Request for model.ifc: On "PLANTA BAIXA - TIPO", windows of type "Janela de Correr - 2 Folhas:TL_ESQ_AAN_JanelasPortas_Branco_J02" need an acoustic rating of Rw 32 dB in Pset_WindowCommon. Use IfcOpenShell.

First a look at what the model holds.

```python
import ifcopenshell
import ifcopenshell.util.element

model = ifcopenshell.open("model.ifc")
print(model.schema)
storey = next(s for s in model.by_type("IfcBuildingStorey") if s.Name == "PLANTA BAIXA - TIPO")
windows = [e for e in ifcopenshell.util.element.get_decomposition(storey) if e.is_a("IfcWindow")]
seen = {}
for e in windows:
    element_type = ifcopenshell.util.element.get_type(e)
    key = (element_type.Name if element_type != e and element_type else None, ifcopenshell.util.element.get_pset(e, "Pset_WindowCommon", "AcousticRating"))
    seen[key] = seen.get(key, 0) + 1
for (name, value), count in sorted(seen.items(), key=str):
    print(count, "x", name, "|", value)
```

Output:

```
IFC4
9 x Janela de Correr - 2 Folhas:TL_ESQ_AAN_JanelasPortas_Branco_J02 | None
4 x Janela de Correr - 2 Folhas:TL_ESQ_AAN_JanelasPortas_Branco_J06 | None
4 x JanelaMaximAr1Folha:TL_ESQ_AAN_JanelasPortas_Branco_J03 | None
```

```python
import ifcopenshell
import ifcopenshell.api.pset
import ifcopenshell.util.element

model = ifcopenshell.open("model.ifc")

storey = next(s for s in model.by_type("IfcBuildingStorey") if s.Name == "PLANTA BAIXA - TIPO")
windows = [e for e in ifcopenshell.util.element.get_decomposition(storey) if e.is_a("IfcWindow")]

count = 0
for e in windows:
    element_type = ifcopenshell.util.element.get_type(e)
    if element_type in (None, e) or element_type.Name != "Janela de Correr - 2 Folhas:TL_ESQ_AAN_JanelasPortas_Branco_J02":
        continue
    # add_pset returns the element's existing set when there is one.
    pset = ifcopenshell.api.pset.add_pset(model, product=e, name="Pset_WindowCommon")
    ifcopenshell.api.pset.edit_pset(model, pset=pset, properties={"AcousticRating": "Rw 32 dB"})
    count += 1

print(count, "windows updated")

model.write("model_v2.ifc")
```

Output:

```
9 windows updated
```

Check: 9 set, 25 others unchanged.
